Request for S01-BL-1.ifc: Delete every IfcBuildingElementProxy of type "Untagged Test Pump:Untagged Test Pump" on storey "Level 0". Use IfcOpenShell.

First a look at what the model holds.

```python
import ifcopenshell
import ifcopenshell.util.element

model = ifcopenshell.open("S01-BL-1.ifc")
print(model.schema)
storey = next(s for s in model.by_type("IfcBuildingStorey") if s.Name == "Level 0")
proxies = [e for e in ifcopenshell.util.element.get_decomposition(storey) if e.is_a("IfcBuildingElementProxy")]
seen = {}
for e in proxies:
    element_type = ifcopenshell.util.element.get_type(e)
    name = element_type.Name if element_type not in (None, e) else None
    seen[name] = seen.get(name, 0) + 1
for name, count in sorted(seen.items(), key=str):
    print(count, "x", name)
```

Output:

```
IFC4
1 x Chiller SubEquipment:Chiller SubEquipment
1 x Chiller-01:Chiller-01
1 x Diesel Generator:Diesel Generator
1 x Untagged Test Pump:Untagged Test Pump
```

```python
import ifcopenshell
import ifcopenshell.api.root
import ifcopenshell.util.element

model = ifcopenshell.open("S01-BL-1.ifc")

storey = next(s for s in model.by_type("IfcBuildingStorey") if s.Name == "Level 0")
proxies = [e for e in ifcopenshell.util.element.get_decomposition(storey) if e.is_a("IfcBuildingElementProxy")]
targets = [e for e in proxies if (t := ifcopenshell.util.element.get_type(e)) not in (None, e) and t.Name == "Untagged Test Pump:Untagged Test Pump"]

for e in targets:
    ifcopenshell.api.root.remove_product(model, product=e)
print(len(targets), "removed")

model.write("S01-BL-1_rev.ifc")
```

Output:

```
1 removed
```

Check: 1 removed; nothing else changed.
